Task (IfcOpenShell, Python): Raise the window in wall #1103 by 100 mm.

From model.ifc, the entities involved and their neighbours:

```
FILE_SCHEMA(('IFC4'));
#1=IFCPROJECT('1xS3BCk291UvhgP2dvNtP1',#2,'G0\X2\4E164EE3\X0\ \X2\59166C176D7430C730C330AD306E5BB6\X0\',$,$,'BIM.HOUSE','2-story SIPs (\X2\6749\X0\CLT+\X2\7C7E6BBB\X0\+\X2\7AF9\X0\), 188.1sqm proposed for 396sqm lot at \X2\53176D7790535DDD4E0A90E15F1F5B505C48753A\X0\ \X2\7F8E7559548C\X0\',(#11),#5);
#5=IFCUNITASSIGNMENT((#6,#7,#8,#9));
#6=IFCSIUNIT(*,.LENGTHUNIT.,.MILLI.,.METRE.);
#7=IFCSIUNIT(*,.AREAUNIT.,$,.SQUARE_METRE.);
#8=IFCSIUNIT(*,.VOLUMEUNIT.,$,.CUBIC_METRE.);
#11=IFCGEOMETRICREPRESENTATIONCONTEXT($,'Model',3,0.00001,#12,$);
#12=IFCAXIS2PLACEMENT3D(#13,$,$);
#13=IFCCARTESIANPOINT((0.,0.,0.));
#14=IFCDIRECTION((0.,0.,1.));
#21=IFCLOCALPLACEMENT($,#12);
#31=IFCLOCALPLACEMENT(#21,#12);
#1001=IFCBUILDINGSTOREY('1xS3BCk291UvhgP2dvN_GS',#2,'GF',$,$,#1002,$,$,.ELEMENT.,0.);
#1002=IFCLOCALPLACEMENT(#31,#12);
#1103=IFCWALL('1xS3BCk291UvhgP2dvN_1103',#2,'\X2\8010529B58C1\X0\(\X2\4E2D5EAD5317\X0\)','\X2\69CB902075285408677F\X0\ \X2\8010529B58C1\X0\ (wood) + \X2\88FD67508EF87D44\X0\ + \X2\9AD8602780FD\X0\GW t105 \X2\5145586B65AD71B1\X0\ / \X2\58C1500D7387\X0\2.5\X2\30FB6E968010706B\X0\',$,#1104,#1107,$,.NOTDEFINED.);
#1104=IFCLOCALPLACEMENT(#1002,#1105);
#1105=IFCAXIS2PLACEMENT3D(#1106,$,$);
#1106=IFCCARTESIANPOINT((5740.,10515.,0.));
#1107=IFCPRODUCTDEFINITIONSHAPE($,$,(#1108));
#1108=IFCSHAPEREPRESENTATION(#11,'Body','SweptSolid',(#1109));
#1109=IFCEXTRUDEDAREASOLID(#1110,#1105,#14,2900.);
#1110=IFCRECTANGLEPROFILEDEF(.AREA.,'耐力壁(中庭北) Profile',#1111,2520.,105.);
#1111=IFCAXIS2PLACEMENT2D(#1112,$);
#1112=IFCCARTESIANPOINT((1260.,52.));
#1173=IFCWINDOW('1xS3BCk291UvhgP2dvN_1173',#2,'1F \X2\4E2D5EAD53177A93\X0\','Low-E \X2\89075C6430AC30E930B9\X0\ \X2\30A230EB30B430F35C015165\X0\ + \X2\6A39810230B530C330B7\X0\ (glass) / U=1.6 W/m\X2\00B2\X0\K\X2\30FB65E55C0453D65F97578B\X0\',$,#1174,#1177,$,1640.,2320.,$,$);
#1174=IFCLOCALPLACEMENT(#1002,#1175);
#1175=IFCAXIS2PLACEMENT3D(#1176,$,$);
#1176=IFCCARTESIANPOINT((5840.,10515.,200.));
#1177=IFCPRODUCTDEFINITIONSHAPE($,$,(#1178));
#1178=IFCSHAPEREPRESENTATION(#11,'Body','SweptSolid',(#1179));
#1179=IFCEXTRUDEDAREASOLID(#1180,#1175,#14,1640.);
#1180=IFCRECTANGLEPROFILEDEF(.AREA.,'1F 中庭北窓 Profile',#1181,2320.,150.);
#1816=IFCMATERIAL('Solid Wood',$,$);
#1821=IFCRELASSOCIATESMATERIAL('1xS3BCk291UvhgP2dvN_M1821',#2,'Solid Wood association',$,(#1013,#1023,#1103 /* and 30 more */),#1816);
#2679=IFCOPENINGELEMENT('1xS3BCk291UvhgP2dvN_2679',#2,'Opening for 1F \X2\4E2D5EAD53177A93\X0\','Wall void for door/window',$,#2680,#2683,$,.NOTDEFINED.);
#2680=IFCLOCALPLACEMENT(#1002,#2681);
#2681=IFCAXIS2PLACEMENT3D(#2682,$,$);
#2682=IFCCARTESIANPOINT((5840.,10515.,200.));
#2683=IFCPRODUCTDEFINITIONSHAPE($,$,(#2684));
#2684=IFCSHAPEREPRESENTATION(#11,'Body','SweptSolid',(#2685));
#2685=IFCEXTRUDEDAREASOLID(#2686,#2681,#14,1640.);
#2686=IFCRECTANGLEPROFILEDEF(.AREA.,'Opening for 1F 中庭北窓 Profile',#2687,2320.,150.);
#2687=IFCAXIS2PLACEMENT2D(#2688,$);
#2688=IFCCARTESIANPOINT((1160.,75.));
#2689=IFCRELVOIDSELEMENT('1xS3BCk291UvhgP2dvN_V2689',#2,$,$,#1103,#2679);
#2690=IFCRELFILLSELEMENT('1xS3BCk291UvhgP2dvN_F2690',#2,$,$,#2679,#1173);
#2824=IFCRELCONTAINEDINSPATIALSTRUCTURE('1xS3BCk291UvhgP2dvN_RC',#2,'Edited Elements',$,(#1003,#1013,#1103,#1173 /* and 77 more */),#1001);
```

```python
import numpy as np
import ifcopenshell
import ifcopenshell.api.geometry
import ifcopenshell.util.placement
import ifcopenshell.util.unit

model = ifcopenshell.open("model.ifc")
unit_scale = ifcopenshell.util.unit.calculate_unit_scale(model)

window = model.by_guid("1xS3BCk291UvhgP2dvN_1173")
opening = window.FillsVoids[0].RelatingOpeningElement
dz = 0.1 / unit_scale

shift = np.array([0.0, 0.0, dz])
# The window is not placed relative to its opening, so move both.
for product in (opening, window):
    matrix = ifcopenshell.util.placement.get_local_placement(product.ObjectPlacement)
    matrix[:3, 3] += shift
    ifcopenshell.api.geometry.edit_object_placement(model, product=product, matrix=matrix, is_si=False)

print(f"moved by {dz * unit_scale:+.3f} m")

model.write("model_updated.ifc")
```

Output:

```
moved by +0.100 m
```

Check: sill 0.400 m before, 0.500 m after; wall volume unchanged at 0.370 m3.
